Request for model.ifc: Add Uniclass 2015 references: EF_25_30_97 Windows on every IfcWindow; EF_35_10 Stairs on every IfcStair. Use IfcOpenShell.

First a look at what the model holds.

```python
import ifcopenshell

model = ifcopenshell.open("model.ifc")
print(model.schema)
print("classifications:", [c.Name for c in model.by_type("IfcClassification")])
for ifc_class in ("IfcDoor", "IfcRoof", "IfcStair", "IfcWall", "IfcWindow"):
    print(ifc_class, len(model.by_type(ifc_class)))
```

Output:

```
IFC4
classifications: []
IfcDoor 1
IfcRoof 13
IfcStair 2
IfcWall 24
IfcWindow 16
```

```python
import ifcopenshell
import ifcopenshell.api.classification

model = ifcopenshell.open("model.ifc")

system = ifcopenshell.api.classification.add_classification(model, classification="Uniclass 2015")

codes = {
    "IfcWindow": ("EF_25_30_97", "Windows"),
    "IfcStair": ("EF_35_10", "Stairs"),
}
for ifc_class, (code, name) in codes.items():
    products = model.by_type(ifc_class)
    ifcopenshell.api.classification.add_reference(
        model, products=products, classification=system, identification=code, name=name
    )
    print(code, len(products))

model.write("model_edited.ifc")
```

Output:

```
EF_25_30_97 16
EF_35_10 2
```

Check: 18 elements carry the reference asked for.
